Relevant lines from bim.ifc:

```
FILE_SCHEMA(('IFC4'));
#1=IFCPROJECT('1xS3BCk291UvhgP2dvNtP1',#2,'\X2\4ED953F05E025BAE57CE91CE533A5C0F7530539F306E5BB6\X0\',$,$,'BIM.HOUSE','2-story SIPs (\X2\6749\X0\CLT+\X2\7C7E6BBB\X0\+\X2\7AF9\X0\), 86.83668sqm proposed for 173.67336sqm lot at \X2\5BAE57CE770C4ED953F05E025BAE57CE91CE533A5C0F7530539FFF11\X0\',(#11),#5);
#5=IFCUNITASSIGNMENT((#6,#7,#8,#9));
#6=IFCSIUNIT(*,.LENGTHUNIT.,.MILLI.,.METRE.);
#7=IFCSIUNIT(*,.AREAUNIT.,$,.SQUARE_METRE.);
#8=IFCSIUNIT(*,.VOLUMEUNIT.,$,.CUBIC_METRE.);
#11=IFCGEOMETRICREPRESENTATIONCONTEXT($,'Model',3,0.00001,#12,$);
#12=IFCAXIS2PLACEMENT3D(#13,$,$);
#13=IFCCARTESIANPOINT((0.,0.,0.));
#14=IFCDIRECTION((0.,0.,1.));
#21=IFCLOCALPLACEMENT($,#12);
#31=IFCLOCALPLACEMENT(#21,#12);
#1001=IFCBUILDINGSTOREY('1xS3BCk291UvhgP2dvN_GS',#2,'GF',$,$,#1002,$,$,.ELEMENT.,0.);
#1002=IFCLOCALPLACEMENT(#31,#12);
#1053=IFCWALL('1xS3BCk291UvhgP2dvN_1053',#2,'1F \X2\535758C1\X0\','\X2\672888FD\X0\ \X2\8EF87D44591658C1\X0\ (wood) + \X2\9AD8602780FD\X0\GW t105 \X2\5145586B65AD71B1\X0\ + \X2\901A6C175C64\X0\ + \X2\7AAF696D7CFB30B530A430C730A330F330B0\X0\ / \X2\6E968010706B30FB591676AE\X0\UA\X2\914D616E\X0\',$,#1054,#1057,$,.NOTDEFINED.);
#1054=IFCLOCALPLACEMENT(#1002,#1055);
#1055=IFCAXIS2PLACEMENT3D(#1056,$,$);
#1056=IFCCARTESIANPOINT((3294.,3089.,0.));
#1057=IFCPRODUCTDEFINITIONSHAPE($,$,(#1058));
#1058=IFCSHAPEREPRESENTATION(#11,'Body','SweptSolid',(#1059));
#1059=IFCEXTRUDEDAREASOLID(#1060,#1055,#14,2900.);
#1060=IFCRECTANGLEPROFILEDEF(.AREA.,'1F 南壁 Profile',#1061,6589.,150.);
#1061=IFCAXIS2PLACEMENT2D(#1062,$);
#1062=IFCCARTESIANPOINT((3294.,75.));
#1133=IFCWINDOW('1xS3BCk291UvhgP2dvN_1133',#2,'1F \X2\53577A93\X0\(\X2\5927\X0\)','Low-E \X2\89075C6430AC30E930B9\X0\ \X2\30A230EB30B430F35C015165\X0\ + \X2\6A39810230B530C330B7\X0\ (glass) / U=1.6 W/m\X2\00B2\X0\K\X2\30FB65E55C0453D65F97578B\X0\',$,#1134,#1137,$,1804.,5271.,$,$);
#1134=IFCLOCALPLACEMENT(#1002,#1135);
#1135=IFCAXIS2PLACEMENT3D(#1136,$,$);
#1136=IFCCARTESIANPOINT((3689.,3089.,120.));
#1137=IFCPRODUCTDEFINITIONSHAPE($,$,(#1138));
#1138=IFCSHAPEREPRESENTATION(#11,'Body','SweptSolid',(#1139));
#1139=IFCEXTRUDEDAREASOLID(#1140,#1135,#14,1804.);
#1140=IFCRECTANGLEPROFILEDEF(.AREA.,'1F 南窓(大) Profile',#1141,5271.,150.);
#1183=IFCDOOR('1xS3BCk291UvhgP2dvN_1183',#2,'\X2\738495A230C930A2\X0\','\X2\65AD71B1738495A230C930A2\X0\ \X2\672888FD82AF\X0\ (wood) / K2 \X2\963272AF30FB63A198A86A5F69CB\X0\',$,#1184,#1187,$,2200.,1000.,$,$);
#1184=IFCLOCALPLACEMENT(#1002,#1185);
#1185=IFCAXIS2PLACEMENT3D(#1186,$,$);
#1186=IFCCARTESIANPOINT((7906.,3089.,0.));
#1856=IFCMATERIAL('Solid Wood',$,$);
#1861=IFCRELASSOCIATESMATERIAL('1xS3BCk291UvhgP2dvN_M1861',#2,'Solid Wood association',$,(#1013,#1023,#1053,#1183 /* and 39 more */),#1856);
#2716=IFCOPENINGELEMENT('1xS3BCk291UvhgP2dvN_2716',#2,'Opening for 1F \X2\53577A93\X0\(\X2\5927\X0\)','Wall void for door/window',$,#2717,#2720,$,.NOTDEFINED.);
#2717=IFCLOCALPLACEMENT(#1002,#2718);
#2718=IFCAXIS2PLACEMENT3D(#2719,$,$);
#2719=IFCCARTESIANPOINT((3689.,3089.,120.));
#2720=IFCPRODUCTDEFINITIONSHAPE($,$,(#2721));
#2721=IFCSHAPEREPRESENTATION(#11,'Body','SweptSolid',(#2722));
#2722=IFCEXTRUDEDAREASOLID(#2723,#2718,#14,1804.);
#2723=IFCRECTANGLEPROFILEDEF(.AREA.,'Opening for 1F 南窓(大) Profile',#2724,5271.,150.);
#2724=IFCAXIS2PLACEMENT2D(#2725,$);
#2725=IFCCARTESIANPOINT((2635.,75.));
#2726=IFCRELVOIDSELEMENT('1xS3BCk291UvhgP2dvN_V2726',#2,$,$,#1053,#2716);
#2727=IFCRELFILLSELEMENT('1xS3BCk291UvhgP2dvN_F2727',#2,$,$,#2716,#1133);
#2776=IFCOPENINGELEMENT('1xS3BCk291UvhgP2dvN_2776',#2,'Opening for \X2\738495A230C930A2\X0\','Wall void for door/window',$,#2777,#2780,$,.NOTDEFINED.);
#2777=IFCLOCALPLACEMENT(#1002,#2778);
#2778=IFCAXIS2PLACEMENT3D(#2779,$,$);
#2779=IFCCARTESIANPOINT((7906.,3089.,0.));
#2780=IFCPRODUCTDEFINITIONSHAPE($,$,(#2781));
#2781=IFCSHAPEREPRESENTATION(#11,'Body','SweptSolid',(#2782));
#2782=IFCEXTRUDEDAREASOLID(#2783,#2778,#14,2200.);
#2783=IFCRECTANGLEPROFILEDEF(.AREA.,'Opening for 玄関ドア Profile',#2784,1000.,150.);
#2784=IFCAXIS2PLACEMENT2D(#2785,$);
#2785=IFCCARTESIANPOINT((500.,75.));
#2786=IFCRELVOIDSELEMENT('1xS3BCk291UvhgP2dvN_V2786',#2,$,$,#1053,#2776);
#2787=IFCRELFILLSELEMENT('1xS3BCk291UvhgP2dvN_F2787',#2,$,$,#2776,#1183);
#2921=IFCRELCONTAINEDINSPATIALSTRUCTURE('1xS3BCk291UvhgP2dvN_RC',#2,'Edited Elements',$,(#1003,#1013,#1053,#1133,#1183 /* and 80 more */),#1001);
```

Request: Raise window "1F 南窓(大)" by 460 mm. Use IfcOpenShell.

```python
import numpy as np
import ifcopenshell
import ifcopenshell.api.geometry
import ifcopenshell.util.placement
import ifcopenshell.util.unit

model = ifcopenshell.open("bim.ifc")
unit_scale = ifcopenshell.util.unit.calculate_unit_scale(model)

window = model.by_id(1133)
opening = window.FillsVoids[0].RelatingOpeningElement
dz = 0.46 / unit_scale

shift = np.array([0.0, 0.0, dz])
# The window is not placed relative to its opening, so move both.
for product in (opening, window):
    matrix = ifcopenshell.util.placement.get_local_placement(product.ObjectPlacement)
    matrix[:3, 3] += shift
    ifcopenshell.api.geometry.edit_object_placement(model, product=product, matrix=matrix, is_si=False)

print(f"moved by {dz * unit_scale:+.3f} m")

model.write("bim_rev.ifc")
```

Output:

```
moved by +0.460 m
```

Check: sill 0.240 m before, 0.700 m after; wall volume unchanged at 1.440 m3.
